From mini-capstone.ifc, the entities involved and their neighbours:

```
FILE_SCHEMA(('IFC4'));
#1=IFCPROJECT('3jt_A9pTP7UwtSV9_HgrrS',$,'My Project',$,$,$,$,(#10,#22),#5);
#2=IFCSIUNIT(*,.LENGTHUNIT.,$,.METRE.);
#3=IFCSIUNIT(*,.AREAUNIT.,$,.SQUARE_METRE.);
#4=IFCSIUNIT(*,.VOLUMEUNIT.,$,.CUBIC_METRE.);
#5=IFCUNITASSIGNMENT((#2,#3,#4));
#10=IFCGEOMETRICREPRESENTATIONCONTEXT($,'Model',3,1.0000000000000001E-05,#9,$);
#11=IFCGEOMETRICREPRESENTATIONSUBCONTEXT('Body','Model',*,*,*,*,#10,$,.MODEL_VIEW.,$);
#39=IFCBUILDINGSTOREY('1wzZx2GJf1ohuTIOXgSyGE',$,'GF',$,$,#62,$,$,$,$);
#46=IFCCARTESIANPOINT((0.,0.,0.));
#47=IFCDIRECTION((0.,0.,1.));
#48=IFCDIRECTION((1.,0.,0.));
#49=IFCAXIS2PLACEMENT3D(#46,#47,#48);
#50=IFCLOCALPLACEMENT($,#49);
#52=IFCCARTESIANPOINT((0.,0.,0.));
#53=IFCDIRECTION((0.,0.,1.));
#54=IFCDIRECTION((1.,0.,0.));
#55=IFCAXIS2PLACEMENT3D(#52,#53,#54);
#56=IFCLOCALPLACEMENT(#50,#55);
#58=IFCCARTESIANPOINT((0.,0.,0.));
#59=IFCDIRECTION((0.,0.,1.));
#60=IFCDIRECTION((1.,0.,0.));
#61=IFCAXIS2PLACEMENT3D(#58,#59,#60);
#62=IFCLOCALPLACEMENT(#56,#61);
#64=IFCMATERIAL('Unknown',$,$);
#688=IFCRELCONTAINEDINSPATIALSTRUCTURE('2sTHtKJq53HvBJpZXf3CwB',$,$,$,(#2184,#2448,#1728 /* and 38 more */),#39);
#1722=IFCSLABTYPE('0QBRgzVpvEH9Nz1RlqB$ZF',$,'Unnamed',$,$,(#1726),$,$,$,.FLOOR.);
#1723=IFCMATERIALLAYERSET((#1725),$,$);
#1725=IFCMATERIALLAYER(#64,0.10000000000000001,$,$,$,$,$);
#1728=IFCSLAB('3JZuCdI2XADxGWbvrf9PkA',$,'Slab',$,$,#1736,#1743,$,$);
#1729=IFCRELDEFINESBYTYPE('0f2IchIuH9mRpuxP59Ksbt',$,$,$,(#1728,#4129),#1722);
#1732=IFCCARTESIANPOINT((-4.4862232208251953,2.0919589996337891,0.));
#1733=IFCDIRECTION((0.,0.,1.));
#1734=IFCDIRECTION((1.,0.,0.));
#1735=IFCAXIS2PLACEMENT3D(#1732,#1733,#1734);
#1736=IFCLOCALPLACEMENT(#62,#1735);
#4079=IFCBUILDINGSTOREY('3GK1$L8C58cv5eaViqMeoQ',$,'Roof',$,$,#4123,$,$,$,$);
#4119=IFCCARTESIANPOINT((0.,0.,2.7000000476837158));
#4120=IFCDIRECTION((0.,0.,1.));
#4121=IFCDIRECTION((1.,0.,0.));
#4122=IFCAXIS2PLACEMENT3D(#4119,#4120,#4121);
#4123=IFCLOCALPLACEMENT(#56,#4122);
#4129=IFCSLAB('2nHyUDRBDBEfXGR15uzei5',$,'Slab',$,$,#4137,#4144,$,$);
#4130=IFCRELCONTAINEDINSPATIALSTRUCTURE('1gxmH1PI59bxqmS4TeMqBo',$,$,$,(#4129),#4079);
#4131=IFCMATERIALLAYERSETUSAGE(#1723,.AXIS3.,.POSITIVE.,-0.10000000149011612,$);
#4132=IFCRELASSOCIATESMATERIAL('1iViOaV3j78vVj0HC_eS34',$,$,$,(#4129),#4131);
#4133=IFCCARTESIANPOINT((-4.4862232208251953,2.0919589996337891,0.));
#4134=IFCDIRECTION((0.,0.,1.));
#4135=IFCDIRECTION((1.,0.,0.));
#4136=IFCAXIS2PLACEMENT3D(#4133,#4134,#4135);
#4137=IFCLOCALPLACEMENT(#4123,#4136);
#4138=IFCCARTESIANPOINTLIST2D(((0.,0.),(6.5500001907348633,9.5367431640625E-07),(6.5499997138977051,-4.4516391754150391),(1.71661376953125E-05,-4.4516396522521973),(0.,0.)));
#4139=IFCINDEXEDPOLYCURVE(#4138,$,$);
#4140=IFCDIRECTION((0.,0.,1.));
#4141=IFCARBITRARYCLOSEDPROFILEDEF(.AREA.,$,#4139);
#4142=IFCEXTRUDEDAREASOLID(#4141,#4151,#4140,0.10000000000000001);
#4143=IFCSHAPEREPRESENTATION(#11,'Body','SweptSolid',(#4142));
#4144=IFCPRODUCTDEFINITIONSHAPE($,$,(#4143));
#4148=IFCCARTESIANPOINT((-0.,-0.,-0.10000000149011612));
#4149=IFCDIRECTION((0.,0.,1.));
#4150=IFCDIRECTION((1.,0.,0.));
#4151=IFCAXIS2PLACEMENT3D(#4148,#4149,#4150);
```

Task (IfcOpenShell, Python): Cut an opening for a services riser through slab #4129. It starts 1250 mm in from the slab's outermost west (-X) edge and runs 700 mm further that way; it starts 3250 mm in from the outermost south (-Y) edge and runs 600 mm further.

```python
import numpy as np
import ifcopenshell
import ifcopenshell.api.feature
import ifcopenshell.api.geometry
import ifcopenshell.api.root
import ifcopenshell.geom
import ifcopenshell.util.placement
import ifcopenshell.util.representation
import ifcopenshell.util.shape
import ifcopenshell.util.unit

model = ifcopenshell.open("mini-capstone.ifc")
unit_scale = ifcopenshell.util.unit.calculate_unit_scale(model)
settings = ifcopenshell.geom.settings()


def volume(element):
    """Net volume in cubic metres, openings subtracted."""
    shape = ifcopenshell.geom.create_shape(settings, element)
    return ifcopenshell.util.shape.get_volume(shape.geometry)


slab = model.by_id(4129)
before = volume(slab)

# Extent in the slab's own axes, in metres. The edges named are its -X and -Y sides.
slab_shape = ifcopenshell.geom.create_shape(settings, slab)
vertices = ifcopenshell.util.shape.get_vertices(slab_shape.geometry)
x_min, y_min, bottom = vertices.min(axis=0)
top = vertices[:, 2].max()

opening = ifcopenshell.api.root.create_entity(model, ifc_class="IfcOpeningElement", name="Services riser opening", predefined_type="OPENING")
context = ifcopenshell.util.representation.get_context(model, "Model", "Body", "MODEL_VIEW")
width, depth = 0.7, 0.6
outline = [(0.0, 0.0), (width, 0.0), (width, depth), (0.0, depth), (0.0, 0.0)]
# Overshoot both faces by 50 mm so the cut is clean.
shape = ifcopenshell.api.geometry.add_slab_representation(
    model, context=context, depth=top - bottom + 0.1, polyline=outline
)
ifcopenshell.api.geometry.assign_representation(model, product=opening, representation=shape)

matrix = ifcopenshell.util.placement.get_local_placement(slab.ObjectPlacement)
matrix[:, 3] = matrix @ np.append(np.array([x_min + 1.25, y_min + 3.25, bottom - 0.05]) / unit_scale, 1.0)
ifcopenshell.api.geometry.edit_object_placement(model, product=opening, matrix=matrix, is_si=False)
ifcopenshell.api.feature.add_feature(model, feature=opening, element=slab)

after = volume(slab)

print(f"slab volume {before:.3f} -> {after:.3f} m3")

model.write("mini-capstone_edited.ifc")
```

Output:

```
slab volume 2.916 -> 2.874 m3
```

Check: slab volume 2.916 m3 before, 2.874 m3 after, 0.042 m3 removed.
